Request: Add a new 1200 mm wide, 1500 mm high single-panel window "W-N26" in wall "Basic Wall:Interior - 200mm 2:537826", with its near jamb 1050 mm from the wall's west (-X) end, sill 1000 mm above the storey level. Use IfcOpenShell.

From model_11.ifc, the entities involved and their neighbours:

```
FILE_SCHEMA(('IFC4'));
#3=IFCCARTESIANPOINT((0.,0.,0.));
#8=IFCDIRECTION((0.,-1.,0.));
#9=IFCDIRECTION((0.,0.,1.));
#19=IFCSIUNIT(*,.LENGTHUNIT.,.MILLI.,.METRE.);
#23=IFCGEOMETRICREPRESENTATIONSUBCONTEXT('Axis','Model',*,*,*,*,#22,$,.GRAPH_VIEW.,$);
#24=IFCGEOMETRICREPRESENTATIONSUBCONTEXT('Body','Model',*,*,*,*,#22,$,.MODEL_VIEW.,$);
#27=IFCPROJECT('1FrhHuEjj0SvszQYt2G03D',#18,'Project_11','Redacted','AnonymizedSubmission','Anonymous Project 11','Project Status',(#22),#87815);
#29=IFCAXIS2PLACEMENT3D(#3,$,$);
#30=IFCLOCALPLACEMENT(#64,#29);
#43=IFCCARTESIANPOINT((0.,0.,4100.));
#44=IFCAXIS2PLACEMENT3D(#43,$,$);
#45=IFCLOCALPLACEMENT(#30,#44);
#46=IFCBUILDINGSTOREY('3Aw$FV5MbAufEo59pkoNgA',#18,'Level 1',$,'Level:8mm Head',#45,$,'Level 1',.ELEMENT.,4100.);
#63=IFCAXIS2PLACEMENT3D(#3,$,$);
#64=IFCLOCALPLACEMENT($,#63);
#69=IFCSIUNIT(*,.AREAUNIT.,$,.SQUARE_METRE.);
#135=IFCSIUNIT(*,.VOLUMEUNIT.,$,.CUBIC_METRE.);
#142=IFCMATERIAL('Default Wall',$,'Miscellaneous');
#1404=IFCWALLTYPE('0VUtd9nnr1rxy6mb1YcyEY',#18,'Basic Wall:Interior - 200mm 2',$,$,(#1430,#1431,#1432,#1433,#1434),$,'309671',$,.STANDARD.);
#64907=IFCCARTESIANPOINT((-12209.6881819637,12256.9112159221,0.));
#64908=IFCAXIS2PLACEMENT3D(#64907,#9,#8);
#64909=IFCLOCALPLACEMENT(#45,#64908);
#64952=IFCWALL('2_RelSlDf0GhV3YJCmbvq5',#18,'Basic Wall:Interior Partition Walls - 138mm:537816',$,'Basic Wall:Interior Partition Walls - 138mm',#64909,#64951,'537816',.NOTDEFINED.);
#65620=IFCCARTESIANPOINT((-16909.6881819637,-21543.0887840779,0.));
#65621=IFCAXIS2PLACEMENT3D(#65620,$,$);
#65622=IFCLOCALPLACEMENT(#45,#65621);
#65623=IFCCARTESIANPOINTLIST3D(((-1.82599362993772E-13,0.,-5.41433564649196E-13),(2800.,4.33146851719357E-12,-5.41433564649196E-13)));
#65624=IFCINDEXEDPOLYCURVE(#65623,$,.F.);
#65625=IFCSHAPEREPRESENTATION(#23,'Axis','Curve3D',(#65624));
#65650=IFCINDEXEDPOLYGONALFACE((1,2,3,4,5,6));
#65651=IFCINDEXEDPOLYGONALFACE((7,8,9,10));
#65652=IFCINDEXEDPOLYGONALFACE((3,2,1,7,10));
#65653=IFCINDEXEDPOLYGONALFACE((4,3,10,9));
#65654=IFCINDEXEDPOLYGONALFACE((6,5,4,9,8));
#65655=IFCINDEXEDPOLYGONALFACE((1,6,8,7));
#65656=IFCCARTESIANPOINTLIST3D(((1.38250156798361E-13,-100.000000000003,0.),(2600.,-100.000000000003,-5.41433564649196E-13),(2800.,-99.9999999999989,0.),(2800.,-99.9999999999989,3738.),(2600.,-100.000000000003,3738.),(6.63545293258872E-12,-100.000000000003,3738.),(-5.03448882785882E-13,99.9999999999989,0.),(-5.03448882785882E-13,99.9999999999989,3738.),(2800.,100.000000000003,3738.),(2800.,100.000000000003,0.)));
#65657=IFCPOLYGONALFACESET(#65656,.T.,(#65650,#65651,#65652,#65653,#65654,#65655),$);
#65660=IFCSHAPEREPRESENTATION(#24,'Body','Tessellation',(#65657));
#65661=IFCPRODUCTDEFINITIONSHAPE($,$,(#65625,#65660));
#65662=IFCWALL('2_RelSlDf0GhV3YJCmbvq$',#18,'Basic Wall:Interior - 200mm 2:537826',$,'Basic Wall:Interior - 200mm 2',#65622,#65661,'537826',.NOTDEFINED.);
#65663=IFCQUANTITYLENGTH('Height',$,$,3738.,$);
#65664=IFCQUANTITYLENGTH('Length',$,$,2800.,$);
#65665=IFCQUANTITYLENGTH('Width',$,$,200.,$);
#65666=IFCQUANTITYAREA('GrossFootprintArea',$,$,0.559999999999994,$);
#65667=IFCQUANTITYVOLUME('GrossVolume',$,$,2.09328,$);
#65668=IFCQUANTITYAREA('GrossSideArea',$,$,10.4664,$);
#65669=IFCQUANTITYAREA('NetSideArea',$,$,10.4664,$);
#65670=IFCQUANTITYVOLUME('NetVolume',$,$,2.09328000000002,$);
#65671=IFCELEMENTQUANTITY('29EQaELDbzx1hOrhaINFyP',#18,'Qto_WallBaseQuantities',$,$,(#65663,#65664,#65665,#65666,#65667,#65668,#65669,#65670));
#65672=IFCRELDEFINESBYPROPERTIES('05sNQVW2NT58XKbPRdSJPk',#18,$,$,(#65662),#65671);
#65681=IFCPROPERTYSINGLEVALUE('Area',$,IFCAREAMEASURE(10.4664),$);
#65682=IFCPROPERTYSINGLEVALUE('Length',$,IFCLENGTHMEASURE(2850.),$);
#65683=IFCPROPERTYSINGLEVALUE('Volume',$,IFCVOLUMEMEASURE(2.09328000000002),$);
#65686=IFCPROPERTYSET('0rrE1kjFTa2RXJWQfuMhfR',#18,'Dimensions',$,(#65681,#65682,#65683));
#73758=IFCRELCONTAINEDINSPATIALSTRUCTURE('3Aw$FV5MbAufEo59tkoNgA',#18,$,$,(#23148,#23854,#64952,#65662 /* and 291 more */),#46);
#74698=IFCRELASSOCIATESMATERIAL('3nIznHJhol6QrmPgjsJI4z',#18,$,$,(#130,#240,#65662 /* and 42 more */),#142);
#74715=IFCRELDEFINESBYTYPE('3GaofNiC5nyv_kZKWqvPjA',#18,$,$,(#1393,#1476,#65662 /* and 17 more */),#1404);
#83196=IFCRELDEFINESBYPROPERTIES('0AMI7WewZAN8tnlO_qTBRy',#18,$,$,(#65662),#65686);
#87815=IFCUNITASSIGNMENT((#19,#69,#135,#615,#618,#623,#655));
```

```python
import numpy as np
import ifcopenshell
import ifcopenshell.api.feature
import ifcopenshell.api.geometry
import ifcopenshell.api.pset
import ifcopenshell.api.root
import ifcopenshell.api.spatial
import ifcopenshell.geom
import ifcopenshell.util.element
import ifcopenshell.util.placement
import ifcopenshell.util.representation
import ifcopenshell.util.shape
import ifcopenshell.util.unit

model = ifcopenshell.open("model_11.ifc")
unit_scale = ifcopenshell.util.unit.calculate_unit_scale(model)
area_scale = ifcopenshell.util.unit.calculate_unit_scale(model, "AREAUNIT")
volume_scale = ifcopenshell.util.unit.calculate_unit_scale(model, "VOLUMEUNIT")
settings = ifcopenshell.geom.settings()


def volume(element):
    """Net volume in cubic metres, openings subtracted."""
    shape = ifcopenshell.geom.create_shape(settings, element)
    return ifcopenshell.util.shape.get_volume(shape.geometry)


wall = model.by_id(65662)
storey = ifcopenshell.util.element.get_container(wall, ifc_class="IfcBuildingStorey")
context = ifcopenshell.util.representation.get_context(model, "Model", "Body", "MODEL_VIEW")
before = volume(wall)

width, height, from_end, sill = 1.2, 1.5, 1.05, 1  # metres

# The wall runs along its own X axis, and the end named is its -X end.
wall_shape = ifcopenshell.geom.create_shape(settings, wall)
x, y, z = ifcopenshell.util.shape.get_vertices(wall_shape.geometry).T
start = x.min() + from_end
face, thickness = float(y.min()), float(y.max() - y.min())
wall_matrix = ifcopenshell.util.placement.get_local_placement(wall.ObjectPlacement)
level = ifcopenshell.util.placement.get_local_placement(storey.ObjectPlacement)[2, 3]


def in_wall(x, y):
    """Placement at x, y metres in the wall's axes, at sill height."""
    matrix = wall_matrix.copy()
    matrix[:, 3] = wall_matrix @ np.array([x / unit_scale, y / unit_scale, 0.0, 1.0])
    matrix[2, 3] = level + sill / unit_scale
    return matrix


# Opening: a box that overshoots both wall faces by 50 mm.
opening = ifcopenshell.api.root.create_entity(model, ifc_class="IfcOpeningElement", predefined_type="OPENING")
box = ifcopenshell.api.geometry.add_wall_representation(
    model, context=context, length=width, height=height, thickness=thickness + 0.1
)
ifcopenshell.api.geometry.assign_representation(model, product=opening, representation=box)
ifcopenshell.api.geometry.edit_object_placement(model, product=opening, matrix=in_wall(start, face - 0.05), is_si=False)
ifcopenshell.api.feature.add_feature(model, feature=opening, element=wall)

window = ifcopenshell.api.root.create_entity(model, ifc_class="IfcWindow", name="W-N26", predefined_type="WINDOW")
window.OverallWidth, window.OverallHeight = width / unit_scale, height / unit_scale
window.PartitioningType = "SINGLE_PANEL"
body = ifcopenshell.api.geometry.add_window_representation(
    model,
    context=context,
    overall_width=window.OverallWidth,
    overall_height=window.OverallHeight,
    partition_type="SINGLE_PANEL",
)
ifcopenshell.api.geometry.assign_representation(model, product=window, representation=body)
ifcopenshell.api.spatial.assign_container(model, products=[window], relating_structure=storey)
ifcopenshell.api.feature.add_filling(model, opening=opening, element=window)

# Centre the window in the wall's thickness.
ifcopenshell.api.geometry.edit_object_placement(model, product=window, matrix=in_wall(start, face), is_si=False)
window_shape = ifcopenshell.geom.create_shape(settings, window)
depth = ifcopenshell.util.shape.get_vertices(window_shape.geometry)[:, 1]
offset = face + thickness / 2 - (depth.min() + depth.max()) / 2
ifcopenshell.api.geometry.edit_object_placement(model, product=window, matrix=in_wall(start, offset), is_si=False)

after = volume(wall)

# Update the wall's stored quantities.
qto = model.by_id(ifcopenshell.util.element.get_pset(wall, "Qto_WallBaseQuantities", should_inherit=False)["id"])
ifcopenshell.api.pset.edit_qto(model, qto=qto, properties={
    "NetSideArea": after / thickness / area_scale,
    "NetVolume": after / volume_scale,
})
pset = model.by_id(ifcopenshell.util.element.get_pset(wall, "Dimensions", should_inherit=False)["id"])
ifcopenshell.api.pset.edit_pset(model, pset=pset, properties={
    "Area": model.create_entity("IfcAreaMeasure", after / thickness / area_scale),
    "Volume": model.create_entity("IfcVolumeMeasure", after / volume_scale),
})

print(f"wall volume {before:.3f} -> {after:.3f} m3")

model.write("model_11_updated.ifc")
```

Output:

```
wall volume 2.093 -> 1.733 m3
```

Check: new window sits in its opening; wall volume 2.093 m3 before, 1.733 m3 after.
